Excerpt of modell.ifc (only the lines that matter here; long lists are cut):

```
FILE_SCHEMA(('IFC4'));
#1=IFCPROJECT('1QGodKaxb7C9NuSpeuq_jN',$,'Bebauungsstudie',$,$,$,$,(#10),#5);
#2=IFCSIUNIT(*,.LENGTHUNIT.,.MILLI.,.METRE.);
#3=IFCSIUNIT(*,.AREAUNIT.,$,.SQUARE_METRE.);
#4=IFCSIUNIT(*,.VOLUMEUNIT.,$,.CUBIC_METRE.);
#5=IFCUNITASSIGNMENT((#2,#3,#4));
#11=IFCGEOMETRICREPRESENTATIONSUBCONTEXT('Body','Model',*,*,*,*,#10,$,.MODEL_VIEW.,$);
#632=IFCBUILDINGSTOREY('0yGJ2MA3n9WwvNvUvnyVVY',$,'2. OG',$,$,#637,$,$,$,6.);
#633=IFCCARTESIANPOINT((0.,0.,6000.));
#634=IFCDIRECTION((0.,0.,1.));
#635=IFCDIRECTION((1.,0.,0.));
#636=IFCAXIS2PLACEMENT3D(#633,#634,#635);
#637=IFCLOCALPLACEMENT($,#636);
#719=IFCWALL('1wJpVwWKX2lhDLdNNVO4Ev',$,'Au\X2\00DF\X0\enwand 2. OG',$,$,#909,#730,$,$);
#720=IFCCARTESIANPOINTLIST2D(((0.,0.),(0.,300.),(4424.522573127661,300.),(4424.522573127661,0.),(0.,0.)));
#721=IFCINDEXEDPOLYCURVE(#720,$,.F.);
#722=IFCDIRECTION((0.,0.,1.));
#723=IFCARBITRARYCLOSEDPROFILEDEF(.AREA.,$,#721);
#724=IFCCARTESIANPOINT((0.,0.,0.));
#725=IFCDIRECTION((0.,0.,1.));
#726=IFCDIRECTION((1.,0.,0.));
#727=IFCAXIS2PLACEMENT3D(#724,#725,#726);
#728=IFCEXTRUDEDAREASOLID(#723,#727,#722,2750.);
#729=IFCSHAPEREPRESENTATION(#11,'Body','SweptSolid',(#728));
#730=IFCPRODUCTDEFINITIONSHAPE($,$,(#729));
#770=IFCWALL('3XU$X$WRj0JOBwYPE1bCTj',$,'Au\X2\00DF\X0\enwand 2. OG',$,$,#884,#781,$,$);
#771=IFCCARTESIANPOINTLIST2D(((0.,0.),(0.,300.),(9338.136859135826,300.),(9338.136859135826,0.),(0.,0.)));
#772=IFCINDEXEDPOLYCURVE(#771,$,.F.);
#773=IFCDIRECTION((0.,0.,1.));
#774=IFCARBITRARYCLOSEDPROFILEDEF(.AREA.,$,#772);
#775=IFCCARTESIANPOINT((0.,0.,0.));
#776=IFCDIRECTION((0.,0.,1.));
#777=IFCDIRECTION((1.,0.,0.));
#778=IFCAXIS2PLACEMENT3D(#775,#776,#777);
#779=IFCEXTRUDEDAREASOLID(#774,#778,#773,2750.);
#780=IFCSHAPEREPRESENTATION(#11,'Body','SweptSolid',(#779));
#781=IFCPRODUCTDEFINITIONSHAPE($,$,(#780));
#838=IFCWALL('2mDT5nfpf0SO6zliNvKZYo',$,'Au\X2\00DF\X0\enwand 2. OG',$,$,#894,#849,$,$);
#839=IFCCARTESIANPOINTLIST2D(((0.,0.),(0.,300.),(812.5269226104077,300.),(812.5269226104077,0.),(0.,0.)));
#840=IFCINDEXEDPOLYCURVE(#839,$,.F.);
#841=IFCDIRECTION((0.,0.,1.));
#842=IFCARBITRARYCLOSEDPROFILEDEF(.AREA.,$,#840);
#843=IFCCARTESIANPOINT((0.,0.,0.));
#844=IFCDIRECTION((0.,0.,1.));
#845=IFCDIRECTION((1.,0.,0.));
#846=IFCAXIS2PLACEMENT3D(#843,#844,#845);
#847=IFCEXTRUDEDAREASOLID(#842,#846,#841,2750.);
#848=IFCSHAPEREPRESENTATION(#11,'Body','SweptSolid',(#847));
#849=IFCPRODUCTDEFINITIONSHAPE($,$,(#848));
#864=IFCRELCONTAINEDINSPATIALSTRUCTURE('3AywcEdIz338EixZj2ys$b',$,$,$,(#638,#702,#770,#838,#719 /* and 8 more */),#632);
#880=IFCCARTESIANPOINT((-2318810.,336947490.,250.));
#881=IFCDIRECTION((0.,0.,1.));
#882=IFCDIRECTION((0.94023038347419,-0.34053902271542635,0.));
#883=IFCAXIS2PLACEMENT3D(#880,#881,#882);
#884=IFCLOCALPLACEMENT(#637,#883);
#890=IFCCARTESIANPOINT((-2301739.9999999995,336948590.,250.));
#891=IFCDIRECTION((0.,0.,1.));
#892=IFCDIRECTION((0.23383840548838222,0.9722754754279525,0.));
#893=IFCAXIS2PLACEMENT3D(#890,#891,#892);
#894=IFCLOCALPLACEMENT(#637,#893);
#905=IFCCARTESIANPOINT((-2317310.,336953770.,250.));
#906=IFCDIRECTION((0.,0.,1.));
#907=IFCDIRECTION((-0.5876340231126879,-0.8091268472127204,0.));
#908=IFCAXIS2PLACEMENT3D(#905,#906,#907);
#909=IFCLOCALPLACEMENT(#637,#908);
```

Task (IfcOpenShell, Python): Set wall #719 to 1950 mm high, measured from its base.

```python
import ifcopenshell
import ifcopenshell.geom
import ifcopenshell.util.representation
import ifcopenshell.util.shape

model = ifcopenshell.open("modell.ifc")
settings = ifcopenshell.geom.settings()


def volume(element):
    """Net volume in cubic metres, openings subtracted."""
    shape = ifcopenshell.geom.create_shape(settings, element)
    return ifcopenshell.util.shape.get_volume(shape.geometry)


wall = model.by_guid("1wJpVwWKX2lhDLdNNVO4Ev")
before = volume(wall)

body = ifcopenshell.util.representation.get_representation(wall, "Model", "Body")
solid = body.Items[0]
old_height = solid.Depth
solid.Depth = 1950.0
after = volume(wall)

print(f"height {old_height:g} -> {solid.Depth:g}, volume {before:.3f} -> {after:.3f} m3")

model.write("modell_updated.ifc")
```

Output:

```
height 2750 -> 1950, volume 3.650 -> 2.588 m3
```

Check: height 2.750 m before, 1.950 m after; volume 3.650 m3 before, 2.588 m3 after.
